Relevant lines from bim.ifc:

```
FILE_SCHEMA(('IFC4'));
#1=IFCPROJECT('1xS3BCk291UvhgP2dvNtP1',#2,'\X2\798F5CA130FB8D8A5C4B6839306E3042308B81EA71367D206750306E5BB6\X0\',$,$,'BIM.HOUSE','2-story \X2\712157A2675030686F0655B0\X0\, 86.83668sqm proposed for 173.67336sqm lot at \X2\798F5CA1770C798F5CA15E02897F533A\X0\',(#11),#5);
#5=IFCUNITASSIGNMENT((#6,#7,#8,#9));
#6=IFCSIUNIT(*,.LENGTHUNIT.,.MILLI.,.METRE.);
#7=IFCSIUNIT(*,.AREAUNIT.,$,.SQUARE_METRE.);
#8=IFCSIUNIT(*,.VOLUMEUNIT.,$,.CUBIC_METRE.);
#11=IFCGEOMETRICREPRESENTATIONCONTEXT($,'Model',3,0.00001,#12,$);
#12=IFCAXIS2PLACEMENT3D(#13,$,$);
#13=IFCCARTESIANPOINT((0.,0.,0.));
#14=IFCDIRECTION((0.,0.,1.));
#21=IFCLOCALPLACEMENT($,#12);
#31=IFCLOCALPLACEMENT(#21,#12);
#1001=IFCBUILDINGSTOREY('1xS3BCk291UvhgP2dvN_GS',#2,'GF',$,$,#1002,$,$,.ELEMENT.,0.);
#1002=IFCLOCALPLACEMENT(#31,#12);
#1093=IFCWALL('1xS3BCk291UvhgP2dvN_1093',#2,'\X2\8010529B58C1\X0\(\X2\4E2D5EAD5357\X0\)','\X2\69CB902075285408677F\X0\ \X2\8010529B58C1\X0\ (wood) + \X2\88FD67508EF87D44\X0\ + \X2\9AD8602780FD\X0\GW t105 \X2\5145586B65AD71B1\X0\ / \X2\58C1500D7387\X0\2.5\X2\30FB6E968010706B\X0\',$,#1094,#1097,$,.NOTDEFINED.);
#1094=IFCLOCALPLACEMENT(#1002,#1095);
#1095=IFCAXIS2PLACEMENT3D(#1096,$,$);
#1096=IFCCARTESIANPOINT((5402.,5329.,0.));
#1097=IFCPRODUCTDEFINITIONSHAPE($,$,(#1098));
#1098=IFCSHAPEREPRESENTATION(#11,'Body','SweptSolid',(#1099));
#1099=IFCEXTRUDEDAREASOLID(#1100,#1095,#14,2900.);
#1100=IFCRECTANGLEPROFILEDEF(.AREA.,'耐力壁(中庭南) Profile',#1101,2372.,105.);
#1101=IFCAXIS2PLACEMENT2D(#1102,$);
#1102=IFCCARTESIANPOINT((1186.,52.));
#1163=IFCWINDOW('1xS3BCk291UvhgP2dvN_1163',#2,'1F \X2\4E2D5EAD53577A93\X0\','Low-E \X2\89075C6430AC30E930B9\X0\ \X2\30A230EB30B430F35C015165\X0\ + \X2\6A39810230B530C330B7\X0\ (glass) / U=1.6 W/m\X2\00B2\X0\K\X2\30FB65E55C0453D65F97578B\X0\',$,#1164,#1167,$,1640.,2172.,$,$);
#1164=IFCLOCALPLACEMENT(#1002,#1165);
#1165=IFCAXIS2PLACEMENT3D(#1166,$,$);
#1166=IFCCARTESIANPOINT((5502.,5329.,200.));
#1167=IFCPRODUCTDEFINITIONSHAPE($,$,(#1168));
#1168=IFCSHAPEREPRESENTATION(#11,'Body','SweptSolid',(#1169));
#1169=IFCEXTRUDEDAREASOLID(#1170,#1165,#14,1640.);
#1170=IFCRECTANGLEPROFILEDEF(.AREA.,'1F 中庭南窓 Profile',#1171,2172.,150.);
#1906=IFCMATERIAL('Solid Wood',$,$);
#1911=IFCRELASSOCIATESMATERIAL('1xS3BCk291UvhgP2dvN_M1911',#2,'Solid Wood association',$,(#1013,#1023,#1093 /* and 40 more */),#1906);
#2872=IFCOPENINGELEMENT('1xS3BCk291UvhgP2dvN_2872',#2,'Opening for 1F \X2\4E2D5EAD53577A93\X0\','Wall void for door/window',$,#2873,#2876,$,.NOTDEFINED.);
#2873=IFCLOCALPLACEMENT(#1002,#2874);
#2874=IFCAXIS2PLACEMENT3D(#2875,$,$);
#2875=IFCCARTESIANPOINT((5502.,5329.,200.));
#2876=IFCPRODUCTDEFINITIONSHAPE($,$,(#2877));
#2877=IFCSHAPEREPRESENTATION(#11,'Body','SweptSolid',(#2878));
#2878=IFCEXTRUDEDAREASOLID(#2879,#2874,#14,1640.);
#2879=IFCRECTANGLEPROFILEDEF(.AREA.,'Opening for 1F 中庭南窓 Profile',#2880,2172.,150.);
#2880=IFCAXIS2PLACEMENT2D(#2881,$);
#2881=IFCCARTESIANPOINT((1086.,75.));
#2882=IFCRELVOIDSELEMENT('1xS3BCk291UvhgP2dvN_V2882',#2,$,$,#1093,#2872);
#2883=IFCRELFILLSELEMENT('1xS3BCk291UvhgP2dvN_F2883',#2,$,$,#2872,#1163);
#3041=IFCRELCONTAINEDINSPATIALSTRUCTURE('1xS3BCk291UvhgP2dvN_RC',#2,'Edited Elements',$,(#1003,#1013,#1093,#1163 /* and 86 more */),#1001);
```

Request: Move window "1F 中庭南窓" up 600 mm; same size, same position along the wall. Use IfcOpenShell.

```python
import numpy as np
import ifcopenshell
import ifcopenshell.api.geometry
import ifcopenshell.util.placement
import ifcopenshell.util.unit

model = ifcopenshell.open("bim.ifc")
unit_scale = ifcopenshell.util.unit.calculate_unit_scale(model)

window = model.by_guid("1xS3BCk291UvhgP2dvN_1163")
opening = window.FillsVoids[0].RelatingOpeningElement
dz = 600.0

shift = np.array([0.0, 0.0, dz])
# The window is not placed relative to its opening, so move both.
for product in (opening, window):
    matrix = ifcopenshell.util.placement.get_local_placement(product.ObjectPlacement)
    matrix[:3, 3] += shift
    ifcopenshell.api.geometry.edit_object_placement(model, product=product, matrix=matrix, is_si=False)

print(f"moved by {dz * unit_scale:+.3f} m")

model.write("bim_v2.ifc")
```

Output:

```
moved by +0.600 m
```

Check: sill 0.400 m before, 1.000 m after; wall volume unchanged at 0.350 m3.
